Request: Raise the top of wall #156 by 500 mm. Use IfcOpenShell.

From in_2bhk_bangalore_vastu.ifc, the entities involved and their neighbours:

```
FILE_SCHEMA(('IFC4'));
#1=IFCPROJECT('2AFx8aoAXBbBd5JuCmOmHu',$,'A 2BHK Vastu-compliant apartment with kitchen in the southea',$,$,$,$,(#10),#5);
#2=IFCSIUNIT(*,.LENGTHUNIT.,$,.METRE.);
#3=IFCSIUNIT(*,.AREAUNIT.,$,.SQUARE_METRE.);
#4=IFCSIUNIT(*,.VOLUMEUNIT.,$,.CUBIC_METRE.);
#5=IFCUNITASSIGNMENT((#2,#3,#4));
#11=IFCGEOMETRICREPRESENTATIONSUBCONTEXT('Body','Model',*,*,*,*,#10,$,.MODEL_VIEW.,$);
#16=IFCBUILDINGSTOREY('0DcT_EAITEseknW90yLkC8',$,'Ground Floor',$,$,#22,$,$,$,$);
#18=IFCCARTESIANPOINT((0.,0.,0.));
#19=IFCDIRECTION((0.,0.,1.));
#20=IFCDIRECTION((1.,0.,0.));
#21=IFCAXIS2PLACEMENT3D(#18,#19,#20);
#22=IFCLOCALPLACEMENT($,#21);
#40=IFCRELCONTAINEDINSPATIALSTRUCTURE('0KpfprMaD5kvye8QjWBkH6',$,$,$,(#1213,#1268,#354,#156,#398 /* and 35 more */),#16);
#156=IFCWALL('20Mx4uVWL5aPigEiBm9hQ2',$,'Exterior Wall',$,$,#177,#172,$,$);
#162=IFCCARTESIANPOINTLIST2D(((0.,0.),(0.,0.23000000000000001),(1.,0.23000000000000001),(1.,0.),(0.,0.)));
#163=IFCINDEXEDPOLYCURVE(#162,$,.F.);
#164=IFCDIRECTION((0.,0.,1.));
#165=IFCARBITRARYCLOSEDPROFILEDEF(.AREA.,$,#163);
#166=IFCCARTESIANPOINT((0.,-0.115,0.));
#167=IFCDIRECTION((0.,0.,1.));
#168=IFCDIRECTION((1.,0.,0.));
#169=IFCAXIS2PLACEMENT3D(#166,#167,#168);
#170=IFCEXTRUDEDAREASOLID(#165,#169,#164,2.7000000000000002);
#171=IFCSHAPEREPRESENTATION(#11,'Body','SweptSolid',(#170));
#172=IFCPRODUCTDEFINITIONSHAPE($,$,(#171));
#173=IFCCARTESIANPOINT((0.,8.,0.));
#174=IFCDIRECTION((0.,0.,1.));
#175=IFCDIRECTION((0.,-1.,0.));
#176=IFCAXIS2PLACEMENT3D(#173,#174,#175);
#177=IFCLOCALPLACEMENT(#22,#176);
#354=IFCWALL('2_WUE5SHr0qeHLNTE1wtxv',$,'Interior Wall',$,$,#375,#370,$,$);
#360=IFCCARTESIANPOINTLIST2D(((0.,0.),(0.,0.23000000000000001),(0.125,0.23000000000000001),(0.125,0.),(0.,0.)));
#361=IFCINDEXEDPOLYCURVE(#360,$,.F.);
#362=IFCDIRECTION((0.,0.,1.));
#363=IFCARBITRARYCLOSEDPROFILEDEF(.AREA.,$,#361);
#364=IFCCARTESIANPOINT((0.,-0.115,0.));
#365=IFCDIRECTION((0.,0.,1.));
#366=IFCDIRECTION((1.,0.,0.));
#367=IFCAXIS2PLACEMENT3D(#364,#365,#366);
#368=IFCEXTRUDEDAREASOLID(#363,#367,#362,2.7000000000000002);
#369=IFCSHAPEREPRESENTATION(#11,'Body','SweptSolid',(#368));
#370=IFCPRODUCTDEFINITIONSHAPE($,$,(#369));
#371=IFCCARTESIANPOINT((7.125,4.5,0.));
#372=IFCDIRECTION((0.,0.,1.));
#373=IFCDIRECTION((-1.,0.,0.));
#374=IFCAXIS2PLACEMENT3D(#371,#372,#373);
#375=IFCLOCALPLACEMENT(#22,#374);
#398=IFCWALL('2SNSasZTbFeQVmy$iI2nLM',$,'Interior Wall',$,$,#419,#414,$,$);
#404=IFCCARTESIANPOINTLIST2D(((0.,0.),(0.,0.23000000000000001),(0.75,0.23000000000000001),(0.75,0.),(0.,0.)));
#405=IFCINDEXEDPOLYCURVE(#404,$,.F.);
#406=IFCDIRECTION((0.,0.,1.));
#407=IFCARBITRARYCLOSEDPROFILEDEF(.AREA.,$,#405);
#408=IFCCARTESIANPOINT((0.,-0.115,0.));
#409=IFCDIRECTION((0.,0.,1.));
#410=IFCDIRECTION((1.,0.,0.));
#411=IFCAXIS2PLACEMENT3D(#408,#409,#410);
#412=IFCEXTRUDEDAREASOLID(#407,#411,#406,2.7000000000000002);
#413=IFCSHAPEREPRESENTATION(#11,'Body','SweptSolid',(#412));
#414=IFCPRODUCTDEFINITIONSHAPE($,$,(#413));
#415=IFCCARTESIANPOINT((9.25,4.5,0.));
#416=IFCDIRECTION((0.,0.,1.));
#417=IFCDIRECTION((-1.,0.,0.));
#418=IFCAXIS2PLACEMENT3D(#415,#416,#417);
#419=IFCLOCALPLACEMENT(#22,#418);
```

```python
import ifcopenshell
import ifcopenshell.geom
import ifcopenshell.util.representation
import ifcopenshell.util.shape
import ifcopenshell.util.unit

model = ifcopenshell.open("in_2bhk_bangalore_vastu.ifc")
unit_scale = ifcopenshell.util.unit.calculate_unit_scale(model)
settings = ifcopenshell.geom.settings()


def volume(element):
    """Net volume in cubic metres, openings subtracted."""
    shape = ifcopenshell.geom.create_shape(settings, element)
    return ifcopenshell.util.shape.get_volume(shape.geometry)


wall = model.by_id(156)
before = volume(wall)

body = ifcopenshell.util.representation.get_representation(wall, "Model", "Body")
solid = body.Items[0]
old_height = solid.Depth
solid.Depth += 0.5 / unit_scale
after = volume(wall)

print(f"height {old_height:g} -> {solid.Depth:g}, volume {before:.3f} -> {after:.3f} m3")

model.write("in_2bhk_bangalore_vastu_updated.ifc")
```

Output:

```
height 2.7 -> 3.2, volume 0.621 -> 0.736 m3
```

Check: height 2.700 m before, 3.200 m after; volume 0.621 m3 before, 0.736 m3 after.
